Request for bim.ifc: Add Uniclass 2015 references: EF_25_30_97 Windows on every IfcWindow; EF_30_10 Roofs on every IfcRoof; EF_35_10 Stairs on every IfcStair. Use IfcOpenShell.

First a look at what the model holds.

```python
import ifcopenshell

model = ifcopenshell.open("bim.ifc")
print(model.schema)
print("classifications:", [c.Name for c in model.by_type("IfcClassification")])
for ifc_class in ("IfcDoor", "IfcRoof", "IfcStair", "IfcWall", "IfcWindow"):
    print(ifc_class, len(model.by_type(ifc_class)))
```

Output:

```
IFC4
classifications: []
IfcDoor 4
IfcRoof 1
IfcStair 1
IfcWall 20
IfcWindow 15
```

```python
import ifcopenshell
import ifcopenshell.api.classification

model = ifcopenshell.open("bim.ifc")

system = ifcopenshell.api.classification.add_classification(model, classification="Uniclass 2015")

codes = {
    "IfcWindow": ("EF_25_30_97", "Windows"),
    "IfcRoof": ("EF_30_10", "Roofs"),
    "IfcStair": ("EF_35_10", "Stairs"),
}
for ifc_class, (code, name) in codes.items():
    products = model.by_type(ifc_class)
    ifcopenshell.api.classification.add_reference(
        model, products=products, classification=system, identification=code, name=name
    )
    print(code, len(products))

model.write("bim_rev.ifc")
```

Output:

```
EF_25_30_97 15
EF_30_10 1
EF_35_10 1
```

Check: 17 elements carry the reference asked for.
